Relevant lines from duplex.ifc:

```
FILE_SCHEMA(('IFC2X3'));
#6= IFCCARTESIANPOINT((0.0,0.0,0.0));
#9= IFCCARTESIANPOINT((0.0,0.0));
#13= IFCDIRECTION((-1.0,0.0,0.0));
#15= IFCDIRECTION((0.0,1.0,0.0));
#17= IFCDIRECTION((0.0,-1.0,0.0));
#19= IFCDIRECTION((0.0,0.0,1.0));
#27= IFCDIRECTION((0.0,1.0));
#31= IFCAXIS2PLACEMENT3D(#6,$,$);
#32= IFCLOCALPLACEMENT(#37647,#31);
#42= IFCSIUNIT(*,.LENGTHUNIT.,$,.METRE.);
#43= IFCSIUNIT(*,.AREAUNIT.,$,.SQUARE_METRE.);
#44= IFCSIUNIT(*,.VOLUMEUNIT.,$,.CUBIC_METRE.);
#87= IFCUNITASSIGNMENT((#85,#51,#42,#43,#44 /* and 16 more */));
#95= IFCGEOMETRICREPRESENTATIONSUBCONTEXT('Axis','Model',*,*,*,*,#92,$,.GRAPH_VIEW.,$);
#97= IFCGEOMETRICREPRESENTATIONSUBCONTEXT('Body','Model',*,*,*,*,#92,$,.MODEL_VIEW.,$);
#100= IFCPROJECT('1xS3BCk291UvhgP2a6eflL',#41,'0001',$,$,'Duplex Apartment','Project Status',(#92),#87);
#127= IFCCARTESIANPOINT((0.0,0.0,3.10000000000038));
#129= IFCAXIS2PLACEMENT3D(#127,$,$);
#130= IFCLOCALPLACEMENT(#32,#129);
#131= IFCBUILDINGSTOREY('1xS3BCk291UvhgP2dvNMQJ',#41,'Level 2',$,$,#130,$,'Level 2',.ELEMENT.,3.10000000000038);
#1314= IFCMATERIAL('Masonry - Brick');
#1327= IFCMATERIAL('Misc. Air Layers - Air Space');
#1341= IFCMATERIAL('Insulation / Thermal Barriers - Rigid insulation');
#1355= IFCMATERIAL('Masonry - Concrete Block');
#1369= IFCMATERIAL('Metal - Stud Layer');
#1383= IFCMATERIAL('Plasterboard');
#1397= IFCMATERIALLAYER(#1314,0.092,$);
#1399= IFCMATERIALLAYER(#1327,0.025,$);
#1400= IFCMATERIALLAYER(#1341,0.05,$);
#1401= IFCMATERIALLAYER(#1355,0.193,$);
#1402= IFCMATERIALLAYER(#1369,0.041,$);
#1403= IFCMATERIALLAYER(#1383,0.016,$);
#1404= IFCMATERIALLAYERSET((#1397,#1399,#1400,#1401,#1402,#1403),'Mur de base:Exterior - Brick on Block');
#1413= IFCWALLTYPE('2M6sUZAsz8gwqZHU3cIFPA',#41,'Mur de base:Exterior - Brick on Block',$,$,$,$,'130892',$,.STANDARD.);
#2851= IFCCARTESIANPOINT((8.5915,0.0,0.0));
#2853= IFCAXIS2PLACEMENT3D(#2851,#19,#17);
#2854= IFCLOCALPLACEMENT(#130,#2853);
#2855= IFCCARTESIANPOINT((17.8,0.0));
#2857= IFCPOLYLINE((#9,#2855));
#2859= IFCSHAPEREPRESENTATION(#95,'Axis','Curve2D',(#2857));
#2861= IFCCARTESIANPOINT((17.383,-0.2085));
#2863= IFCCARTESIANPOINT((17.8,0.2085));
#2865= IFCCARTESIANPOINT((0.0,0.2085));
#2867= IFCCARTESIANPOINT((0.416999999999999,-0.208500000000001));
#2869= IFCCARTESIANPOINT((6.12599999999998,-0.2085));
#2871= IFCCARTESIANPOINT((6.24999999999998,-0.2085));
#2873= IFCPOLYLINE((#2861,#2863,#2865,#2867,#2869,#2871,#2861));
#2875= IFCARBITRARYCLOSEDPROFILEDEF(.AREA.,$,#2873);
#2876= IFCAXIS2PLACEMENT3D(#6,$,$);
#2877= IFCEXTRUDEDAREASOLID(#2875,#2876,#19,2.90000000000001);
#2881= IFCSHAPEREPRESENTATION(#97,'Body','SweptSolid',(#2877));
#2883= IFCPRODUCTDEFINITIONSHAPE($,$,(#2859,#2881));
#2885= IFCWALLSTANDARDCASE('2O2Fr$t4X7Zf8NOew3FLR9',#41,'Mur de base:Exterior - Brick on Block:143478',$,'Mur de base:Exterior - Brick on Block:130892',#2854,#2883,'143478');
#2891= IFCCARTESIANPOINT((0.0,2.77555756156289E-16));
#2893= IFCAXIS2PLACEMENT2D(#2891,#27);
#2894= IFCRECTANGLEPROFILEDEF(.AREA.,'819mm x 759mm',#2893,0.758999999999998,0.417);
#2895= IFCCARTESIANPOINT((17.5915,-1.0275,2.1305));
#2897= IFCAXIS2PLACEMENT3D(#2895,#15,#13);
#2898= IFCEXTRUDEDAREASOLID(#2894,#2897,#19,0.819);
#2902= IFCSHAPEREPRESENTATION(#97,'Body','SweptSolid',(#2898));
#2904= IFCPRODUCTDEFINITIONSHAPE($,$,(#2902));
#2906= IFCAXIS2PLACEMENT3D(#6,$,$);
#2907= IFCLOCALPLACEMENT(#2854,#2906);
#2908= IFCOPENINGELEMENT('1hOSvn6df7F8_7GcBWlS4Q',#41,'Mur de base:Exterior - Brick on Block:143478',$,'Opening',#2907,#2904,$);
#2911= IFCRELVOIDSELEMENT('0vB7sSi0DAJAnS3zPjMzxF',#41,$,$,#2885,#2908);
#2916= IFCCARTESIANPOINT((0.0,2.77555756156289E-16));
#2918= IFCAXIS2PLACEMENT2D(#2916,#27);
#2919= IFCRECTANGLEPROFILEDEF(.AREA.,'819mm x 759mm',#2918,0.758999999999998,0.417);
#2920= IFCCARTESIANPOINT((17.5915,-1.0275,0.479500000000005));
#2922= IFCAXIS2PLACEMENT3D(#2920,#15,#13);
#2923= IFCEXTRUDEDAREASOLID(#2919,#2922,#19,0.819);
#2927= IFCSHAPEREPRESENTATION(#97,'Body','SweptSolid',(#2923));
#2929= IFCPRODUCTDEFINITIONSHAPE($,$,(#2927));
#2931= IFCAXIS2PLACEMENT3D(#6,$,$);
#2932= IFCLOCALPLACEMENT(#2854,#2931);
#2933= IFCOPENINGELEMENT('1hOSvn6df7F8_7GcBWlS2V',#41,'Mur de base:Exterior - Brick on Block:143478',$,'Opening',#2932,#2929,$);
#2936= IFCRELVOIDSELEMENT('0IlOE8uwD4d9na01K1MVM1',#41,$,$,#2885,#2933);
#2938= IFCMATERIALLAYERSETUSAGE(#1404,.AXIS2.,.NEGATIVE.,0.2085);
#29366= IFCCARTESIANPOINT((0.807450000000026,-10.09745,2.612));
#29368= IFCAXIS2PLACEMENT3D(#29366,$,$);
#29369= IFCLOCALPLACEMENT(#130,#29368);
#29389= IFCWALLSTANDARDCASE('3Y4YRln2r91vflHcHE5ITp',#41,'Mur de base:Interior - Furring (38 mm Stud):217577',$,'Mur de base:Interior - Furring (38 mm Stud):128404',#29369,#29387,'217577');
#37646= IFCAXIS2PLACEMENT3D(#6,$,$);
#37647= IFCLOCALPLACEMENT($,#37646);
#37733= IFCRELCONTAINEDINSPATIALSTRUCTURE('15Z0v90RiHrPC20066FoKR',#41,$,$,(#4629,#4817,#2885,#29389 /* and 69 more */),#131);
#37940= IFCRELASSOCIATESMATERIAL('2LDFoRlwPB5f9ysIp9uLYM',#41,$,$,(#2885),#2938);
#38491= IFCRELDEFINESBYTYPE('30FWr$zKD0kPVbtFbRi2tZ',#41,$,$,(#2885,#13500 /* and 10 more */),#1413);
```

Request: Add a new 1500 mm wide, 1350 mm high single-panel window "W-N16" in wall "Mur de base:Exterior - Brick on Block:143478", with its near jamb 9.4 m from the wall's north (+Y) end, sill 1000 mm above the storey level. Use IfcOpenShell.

```python
import numpy as np
import ifcopenshell
import ifcopenshell.api.feature
import ifcopenshell.api.geometry
import ifcopenshell.api.root
import ifcopenshell.api.spatial
import ifcopenshell.api.type
import ifcopenshell.geom
import ifcopenshell.util.element
import ifcopenshell.util.placement
import ifcopenshell.util.representation
import ifcopenshell.util.shape
import ifcopenshell.util.unit

model = ifcopenshell.open("duplex.ifc")
unit_scale = ifcopenshell.util.unit.calculate_unit_scale(model)
settings = ifcopenshell.geom.settings()


def volume(element):
    """Net volume in cubic metres, openings subtracted."""
    shape = ifcopenshell.geom.create_shape(settings, element)
    return ifcopenshell.util.shape.get_volume(shape.geometry)


wall = model.by_guid("2O2Fr$t4X7Zf8NOew3FLR9")
storey = ifcopenshell.util.element.get_container(wall, ifc_class="IfcBuildingStorey")
context = ifcopenshell.util.representation.get_context(model, "Model", "Body", "MODEL_VIEW")
before = volume(wall)

width, height, from_end, sill = 1.5, 1.35, 9.4, 1  # metres

# The wall runs along its own X axis, and the end named is its -X end.
wall_shape = ifcopenshell.geom.create_shape(settings, wall)
x, y, z = ifcopenshell.util.shape.get_vertices(wall_shape.geometry).T
start = x.min() + from_end
face, thickness = float(y.min()), float(y.max() - y.min())
wall_matrix = ifcopenshell.util.placement.get_local_placement(wall.ObjectPlacement)
level = ifcopenshell.util.placement.get_local_placement(storey.ObjectPlacement)[2, 3]


def in_wall(x, y):
    """Placement at x, y metres in the wall's axes, at sill height."""
    matrix = wall_matrix.copy()
    matrix[:, 3] = wall_matrix @ np.array([x / unit_scale, y / unit_scale, 0.0, 1.0])
    matrix[2, 3] = level + sill / unit_scale
    return matrix


# Opening: a box that overshoots both wall faces by 50 mm.
opening = ifcopenshell.api.root.create_entity(model, ifc_class="IfcOpeningElement")
box = ifcopenshell.api.geometry.add_wall_representation(
    model, context=context, length=width, height=height, thickness=thickness + 0.1
)
ifcopenshell.api.geometry.assign_representation(model, product=opening, representation=box)
ifcopenshell.api.geometry.edit_object_placement(model, product=opening, matrix=in_wall(start, face - 0.05), is_si=False)
ifcopenshell.api.feature.add_feature(model, feature=opening, element=wall)

window = ifcopenshell.api.root.create_entity(model, ifc_class="IfcWindow", name="W-N16")
window.OverallWidth, window.OverallHeight = width / unit_scale, height / unit_scale
body = ifcopenshell.api.geometry.add_window_representation(
    model,
    context=context,
    overall_width=window.OverallWidth,
    overall_height=window.OverallHeight,
    partition_type="SINGLE_PANEL",
)
ifcopenshell.api.geometry.assign_representation(model, product=window, representation=body)
ifcopenshell.api.spatial.assign_container(model, products=[window], relating_structure=storey)
fills = ifcopenshell.api.feature.add_filling(model, opening=opening, element=window)
fills.OwnerHistory = window.OwnerHistory  # required in IFC2X3

# IFC2X3 keeps the operation on the window style.
style = ifcopenshell.api.root.create_entity(model, ifc_class="IfcWindowStyle", name="W-N16")
style.OperationType, style.ConstructionType = "SINGLE_PANEL", "NOTDEFINED"
style.ParameterTakesPrecedence = style.Sizeable = False
ifcopenshell.api.type.assign_type(model, related_objects=[window], relating_type=style)

# Centre the window in the wall's thickness.
ifcopenshell.api.geometry.edit_object_placement(model, product=window, matrix=in_wall(start, face), is_si=False)
window_shape = ifcopenshell.geom.create_shape(settings, window)
depth = ifcopenshell.util.shape.get_vertices(window_shape.geometry)[:, 1]
offset = face + thickness / 2 - (depth.min() + depth.max()) / 2
ifcopenshell.api.geometry.edit_object_placement(model, product=window, matrix=in_wall(start, offset), is_si=False)

after = volume(wall)

print(f"wall volume {before:.3f} -> {after:.3f} m3")

model.write("duplex_v2.ifc")
```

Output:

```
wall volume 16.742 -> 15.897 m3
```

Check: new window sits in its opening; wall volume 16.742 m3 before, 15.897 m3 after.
